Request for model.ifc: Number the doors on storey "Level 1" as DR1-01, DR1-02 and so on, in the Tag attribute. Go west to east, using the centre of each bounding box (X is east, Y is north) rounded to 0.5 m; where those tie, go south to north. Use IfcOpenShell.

First a look at what the model holds.

```python
import ifcopenshell
import ifcopenshell.util.element
import ifcopenshell.util.placement

model = ifcopenshell.open("model.ifc")
print(model.schema)
storey = next(s for s in model.by_type("IfcBuildingStorey") if s.Name == "Level 1")
doors = [e for e in ifcopenshell.util.element.get_decomposition(storey) if e.is_a("IfcDoor")]
for e in sorted(doors, key=lambda e: e.id()):
    origin = ifcopenshell.util.placement.get_local_placement(e.ObjectPlacement)[:3, 3]
    print(e.id(), e.Tag, e.Name, origin.round(2) + 0.0, sep=" | ")
```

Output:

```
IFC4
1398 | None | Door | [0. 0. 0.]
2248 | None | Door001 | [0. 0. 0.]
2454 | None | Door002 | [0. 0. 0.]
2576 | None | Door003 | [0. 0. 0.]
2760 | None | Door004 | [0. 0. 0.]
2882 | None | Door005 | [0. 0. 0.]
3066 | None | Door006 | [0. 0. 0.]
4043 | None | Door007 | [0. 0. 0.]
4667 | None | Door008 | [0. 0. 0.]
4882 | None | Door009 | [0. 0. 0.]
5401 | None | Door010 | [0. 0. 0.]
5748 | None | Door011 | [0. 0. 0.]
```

```python
import ifcopenshell
import ifcopenshell.geom
import ifcopenshell.util.element
import ifcopenshell.util.shape

model = ifcopenshell.open("model.ifc")
settings = ifcopenshell.geom.settings()
settings.set("use-world-coords", True)


def centre(element):
    shape = ifcopenshell.geom.create_shape(settings, element)
    return ifcopenshell.util.shape.get_bbox_centroid(shape.geometry)


storey = next(s for s in model.by_type("IfcBuildingStorey") if s.Name == "Level 1")
doors = [e for e in ifcopenshell.util.element.get_decomposition(storey) if e.is_a("IfcDoor")]

# Insertion points can sit at a corner or the storey origin, so sort by the geometry (in metres).
centres = {e: centre(e) for e in doors}
doors.sort(key=lambda e: (round(centres[e][0] / 0.5), centres[e][1]))

for i, e in enumerate(doors, start=1):
    number = f"DR1-{i:02d}"
    e.Tag = number
    print(e.id(), number)

model.write("model_v2.ifc")
```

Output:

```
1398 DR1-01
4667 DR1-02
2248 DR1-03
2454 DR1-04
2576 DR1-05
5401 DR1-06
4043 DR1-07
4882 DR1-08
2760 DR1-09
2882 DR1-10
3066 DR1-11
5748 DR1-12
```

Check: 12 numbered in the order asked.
